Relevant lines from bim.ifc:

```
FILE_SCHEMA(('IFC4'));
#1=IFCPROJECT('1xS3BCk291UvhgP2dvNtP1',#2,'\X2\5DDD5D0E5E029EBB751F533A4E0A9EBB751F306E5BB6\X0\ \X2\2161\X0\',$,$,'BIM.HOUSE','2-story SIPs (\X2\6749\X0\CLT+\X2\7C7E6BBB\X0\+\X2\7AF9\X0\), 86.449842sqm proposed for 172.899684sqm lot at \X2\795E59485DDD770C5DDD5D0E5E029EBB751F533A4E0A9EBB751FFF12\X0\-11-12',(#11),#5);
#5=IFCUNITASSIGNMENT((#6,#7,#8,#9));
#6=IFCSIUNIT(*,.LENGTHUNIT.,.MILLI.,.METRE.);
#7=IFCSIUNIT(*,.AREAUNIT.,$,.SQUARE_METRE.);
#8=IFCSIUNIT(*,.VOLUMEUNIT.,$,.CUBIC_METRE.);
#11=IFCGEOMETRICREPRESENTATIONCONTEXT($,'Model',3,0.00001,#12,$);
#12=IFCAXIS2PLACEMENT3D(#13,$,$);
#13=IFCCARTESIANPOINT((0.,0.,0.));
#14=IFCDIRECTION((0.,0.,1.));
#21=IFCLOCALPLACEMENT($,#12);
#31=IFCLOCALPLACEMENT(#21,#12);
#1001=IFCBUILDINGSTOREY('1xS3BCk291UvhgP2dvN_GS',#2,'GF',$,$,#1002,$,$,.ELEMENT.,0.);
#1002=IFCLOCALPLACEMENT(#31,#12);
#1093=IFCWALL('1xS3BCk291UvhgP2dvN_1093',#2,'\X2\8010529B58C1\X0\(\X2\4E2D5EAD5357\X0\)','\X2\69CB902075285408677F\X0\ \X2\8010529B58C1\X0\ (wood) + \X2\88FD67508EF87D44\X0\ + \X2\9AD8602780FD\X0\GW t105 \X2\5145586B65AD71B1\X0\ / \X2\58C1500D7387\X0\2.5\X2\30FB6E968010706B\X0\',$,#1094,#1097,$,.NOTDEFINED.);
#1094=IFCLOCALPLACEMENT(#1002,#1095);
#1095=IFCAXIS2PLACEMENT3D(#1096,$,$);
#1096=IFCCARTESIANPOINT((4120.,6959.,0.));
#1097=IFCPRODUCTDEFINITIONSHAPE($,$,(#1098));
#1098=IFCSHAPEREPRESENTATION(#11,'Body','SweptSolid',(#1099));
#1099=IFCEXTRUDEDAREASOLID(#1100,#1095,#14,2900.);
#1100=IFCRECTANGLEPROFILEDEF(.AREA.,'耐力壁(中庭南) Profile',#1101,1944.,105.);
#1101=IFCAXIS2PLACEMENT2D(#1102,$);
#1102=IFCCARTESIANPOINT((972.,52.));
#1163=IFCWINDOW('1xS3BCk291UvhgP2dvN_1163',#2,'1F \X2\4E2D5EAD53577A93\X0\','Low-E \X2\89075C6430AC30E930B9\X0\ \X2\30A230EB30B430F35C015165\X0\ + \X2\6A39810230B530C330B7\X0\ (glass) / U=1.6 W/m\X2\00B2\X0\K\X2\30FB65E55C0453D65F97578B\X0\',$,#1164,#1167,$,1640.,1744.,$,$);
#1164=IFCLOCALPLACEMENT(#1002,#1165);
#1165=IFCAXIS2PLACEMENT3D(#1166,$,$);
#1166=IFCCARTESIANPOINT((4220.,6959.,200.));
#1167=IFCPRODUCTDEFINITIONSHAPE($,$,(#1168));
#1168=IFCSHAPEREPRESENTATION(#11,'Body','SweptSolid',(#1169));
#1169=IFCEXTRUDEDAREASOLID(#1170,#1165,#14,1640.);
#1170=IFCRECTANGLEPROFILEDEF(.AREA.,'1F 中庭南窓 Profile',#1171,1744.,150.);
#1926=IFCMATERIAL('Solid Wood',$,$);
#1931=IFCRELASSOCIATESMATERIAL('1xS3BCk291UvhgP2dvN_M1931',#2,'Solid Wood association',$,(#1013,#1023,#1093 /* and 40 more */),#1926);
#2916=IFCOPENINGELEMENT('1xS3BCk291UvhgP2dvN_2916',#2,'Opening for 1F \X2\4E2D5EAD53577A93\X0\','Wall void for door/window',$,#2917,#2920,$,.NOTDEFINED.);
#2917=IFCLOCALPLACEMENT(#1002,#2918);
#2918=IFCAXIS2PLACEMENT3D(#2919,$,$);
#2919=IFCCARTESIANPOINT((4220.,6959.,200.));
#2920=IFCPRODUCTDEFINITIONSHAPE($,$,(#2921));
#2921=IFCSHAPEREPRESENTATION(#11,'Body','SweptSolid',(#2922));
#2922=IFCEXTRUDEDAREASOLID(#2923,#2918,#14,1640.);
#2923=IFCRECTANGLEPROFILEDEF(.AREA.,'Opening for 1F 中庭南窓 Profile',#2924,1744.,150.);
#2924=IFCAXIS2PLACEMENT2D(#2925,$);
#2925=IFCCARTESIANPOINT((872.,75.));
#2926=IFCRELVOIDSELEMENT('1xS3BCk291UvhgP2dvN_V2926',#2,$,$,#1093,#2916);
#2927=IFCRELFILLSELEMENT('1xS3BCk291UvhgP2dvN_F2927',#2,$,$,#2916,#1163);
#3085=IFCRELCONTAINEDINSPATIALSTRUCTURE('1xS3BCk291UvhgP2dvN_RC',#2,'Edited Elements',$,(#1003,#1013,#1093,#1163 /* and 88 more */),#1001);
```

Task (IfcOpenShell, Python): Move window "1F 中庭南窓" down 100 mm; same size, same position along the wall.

```python
import numpy as np
import ifcopenshell
import ifcopenshell.api.geometry
import ifcopenshell.util.placement
import ifcopenshell.util.unit

model = ifcopenshell.open("bim.ifc")
unit_scale = ifcopenshell.util.unit.calculate_unit_scale(model)

window = model.by_guid("1xS3BCk291UvhgP2dvN_1163")
opening = window.FillsVoids[0].RelatingOpeningElement
dz = -100.0

shift = np.array([0.0, 0.0, dz])
# The window is not placed relative to its opening, so move both.
for product in (opening, window):
    matrix = ifcopenshell.util.placement.get_local_placement(product.ObjectPlacement)
    matrix[:3, 3] += shift
    ifcopenshell.api.geometry.edit_object_placement(model, product=product, matrix=matrix, is_si=False)

print(f"moved by {dz * unit_scale:+.3f} m")

model.write("bim_rev.ifc")
```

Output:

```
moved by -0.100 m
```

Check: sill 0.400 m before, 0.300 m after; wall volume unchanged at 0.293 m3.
